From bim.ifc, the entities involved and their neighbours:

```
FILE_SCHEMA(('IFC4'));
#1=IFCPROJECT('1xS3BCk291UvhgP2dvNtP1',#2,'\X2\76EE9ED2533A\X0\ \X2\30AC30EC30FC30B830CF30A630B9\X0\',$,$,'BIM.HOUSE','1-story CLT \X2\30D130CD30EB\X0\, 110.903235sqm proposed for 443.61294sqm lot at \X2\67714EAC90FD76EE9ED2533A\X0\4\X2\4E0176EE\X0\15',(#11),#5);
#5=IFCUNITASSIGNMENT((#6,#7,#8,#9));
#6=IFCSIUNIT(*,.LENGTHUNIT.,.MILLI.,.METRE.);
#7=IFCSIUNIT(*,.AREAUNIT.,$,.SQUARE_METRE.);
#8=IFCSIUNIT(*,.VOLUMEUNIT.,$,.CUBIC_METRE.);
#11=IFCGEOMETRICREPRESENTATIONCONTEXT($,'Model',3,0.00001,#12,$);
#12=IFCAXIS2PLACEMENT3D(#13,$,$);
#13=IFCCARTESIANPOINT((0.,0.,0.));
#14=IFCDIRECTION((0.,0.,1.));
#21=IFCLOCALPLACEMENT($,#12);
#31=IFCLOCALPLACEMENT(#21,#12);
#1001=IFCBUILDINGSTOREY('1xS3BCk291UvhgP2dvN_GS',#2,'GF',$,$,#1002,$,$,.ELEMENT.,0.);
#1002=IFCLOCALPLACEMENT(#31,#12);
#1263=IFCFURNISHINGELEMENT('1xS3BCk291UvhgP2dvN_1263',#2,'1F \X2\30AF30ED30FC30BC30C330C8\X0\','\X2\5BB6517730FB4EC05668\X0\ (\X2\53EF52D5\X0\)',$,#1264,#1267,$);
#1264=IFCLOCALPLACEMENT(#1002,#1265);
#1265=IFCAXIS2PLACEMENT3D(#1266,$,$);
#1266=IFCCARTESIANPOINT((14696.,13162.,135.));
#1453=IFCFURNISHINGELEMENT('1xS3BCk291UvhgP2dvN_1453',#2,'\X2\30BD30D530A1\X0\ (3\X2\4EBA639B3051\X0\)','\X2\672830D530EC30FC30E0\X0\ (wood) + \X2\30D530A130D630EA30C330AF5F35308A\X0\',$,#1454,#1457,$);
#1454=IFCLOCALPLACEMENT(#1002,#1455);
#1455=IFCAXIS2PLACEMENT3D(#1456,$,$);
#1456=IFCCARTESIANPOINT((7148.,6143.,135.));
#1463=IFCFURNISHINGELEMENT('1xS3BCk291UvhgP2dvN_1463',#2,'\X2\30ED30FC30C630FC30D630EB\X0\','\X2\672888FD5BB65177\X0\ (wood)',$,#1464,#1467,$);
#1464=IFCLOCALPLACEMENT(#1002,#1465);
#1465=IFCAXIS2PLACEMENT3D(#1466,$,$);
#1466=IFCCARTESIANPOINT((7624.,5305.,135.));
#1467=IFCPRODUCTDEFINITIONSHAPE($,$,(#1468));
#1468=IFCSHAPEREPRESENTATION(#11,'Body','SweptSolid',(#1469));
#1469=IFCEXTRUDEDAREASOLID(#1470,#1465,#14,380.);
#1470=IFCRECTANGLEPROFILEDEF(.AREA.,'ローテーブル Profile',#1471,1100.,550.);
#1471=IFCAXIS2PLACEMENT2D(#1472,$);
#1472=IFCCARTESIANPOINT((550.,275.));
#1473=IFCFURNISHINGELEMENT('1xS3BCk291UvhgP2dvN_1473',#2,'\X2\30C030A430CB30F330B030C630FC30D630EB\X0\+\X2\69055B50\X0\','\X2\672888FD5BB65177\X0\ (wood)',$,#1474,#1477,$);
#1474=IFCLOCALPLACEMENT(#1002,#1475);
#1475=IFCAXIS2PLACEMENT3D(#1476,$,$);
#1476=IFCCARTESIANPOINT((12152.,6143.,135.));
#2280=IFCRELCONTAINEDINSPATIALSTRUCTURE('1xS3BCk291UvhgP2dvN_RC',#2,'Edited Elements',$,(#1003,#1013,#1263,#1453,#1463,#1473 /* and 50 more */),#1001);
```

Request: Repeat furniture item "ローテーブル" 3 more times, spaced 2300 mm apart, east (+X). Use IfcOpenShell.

```python
import numpy as np
import ifcopenshell
import ifcopenshell.api.geometry
import ifcopenshell.api.root
import ifcopenshell.util.element
import ifcopenshell.util.placement

model = ifcopenshell.open("bim.ifc")


def reuse_history(source, copy):
    """copy_class also copies each property set's owner history, people and application; keep the originals."""
    for rel in copy.IsDefinedBy:
        if rel.is_a("IfcRelDefinesByProperties") and (history := rel.RelatingPropertyDefinition.OwnerHistory):
            rel.RelatingPropertyDefinition.OwnerHistory = source.OwnerHistory
            ifcopenshell.util.element.remove_deep2(model, history)


source = model.by_id(1463)
base = ifcopenshell.util.placement.get_local_placement(source.ObjectPlacement)
step = np.array([1.0, 0.0, 0.0]) * 2300.0

for i in range(1, 4):
    copy = ifcopenshell.api.root.copy_class(model, product=source)
    copy.Representation = ifcopenshell.util.element.copy_deep(
        model, source.Representation, exclude=["IfcGeometricRepresentationContext", "IfcRepresentationMap"]
    )
    reuse_history(source, copy)
    matrix = base.copy()
    matrix[:3, 3] += i * step
    print("added at", matrix[:3, 3].round(3) + 0.0)
    ifcopenshell.api.geometry.edit_object_placement(model, product=copy, matrix=matrix, is_si=False)

model.write("bim_updated.ifc")
```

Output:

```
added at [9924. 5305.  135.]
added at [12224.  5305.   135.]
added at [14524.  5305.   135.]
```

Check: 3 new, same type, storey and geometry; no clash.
